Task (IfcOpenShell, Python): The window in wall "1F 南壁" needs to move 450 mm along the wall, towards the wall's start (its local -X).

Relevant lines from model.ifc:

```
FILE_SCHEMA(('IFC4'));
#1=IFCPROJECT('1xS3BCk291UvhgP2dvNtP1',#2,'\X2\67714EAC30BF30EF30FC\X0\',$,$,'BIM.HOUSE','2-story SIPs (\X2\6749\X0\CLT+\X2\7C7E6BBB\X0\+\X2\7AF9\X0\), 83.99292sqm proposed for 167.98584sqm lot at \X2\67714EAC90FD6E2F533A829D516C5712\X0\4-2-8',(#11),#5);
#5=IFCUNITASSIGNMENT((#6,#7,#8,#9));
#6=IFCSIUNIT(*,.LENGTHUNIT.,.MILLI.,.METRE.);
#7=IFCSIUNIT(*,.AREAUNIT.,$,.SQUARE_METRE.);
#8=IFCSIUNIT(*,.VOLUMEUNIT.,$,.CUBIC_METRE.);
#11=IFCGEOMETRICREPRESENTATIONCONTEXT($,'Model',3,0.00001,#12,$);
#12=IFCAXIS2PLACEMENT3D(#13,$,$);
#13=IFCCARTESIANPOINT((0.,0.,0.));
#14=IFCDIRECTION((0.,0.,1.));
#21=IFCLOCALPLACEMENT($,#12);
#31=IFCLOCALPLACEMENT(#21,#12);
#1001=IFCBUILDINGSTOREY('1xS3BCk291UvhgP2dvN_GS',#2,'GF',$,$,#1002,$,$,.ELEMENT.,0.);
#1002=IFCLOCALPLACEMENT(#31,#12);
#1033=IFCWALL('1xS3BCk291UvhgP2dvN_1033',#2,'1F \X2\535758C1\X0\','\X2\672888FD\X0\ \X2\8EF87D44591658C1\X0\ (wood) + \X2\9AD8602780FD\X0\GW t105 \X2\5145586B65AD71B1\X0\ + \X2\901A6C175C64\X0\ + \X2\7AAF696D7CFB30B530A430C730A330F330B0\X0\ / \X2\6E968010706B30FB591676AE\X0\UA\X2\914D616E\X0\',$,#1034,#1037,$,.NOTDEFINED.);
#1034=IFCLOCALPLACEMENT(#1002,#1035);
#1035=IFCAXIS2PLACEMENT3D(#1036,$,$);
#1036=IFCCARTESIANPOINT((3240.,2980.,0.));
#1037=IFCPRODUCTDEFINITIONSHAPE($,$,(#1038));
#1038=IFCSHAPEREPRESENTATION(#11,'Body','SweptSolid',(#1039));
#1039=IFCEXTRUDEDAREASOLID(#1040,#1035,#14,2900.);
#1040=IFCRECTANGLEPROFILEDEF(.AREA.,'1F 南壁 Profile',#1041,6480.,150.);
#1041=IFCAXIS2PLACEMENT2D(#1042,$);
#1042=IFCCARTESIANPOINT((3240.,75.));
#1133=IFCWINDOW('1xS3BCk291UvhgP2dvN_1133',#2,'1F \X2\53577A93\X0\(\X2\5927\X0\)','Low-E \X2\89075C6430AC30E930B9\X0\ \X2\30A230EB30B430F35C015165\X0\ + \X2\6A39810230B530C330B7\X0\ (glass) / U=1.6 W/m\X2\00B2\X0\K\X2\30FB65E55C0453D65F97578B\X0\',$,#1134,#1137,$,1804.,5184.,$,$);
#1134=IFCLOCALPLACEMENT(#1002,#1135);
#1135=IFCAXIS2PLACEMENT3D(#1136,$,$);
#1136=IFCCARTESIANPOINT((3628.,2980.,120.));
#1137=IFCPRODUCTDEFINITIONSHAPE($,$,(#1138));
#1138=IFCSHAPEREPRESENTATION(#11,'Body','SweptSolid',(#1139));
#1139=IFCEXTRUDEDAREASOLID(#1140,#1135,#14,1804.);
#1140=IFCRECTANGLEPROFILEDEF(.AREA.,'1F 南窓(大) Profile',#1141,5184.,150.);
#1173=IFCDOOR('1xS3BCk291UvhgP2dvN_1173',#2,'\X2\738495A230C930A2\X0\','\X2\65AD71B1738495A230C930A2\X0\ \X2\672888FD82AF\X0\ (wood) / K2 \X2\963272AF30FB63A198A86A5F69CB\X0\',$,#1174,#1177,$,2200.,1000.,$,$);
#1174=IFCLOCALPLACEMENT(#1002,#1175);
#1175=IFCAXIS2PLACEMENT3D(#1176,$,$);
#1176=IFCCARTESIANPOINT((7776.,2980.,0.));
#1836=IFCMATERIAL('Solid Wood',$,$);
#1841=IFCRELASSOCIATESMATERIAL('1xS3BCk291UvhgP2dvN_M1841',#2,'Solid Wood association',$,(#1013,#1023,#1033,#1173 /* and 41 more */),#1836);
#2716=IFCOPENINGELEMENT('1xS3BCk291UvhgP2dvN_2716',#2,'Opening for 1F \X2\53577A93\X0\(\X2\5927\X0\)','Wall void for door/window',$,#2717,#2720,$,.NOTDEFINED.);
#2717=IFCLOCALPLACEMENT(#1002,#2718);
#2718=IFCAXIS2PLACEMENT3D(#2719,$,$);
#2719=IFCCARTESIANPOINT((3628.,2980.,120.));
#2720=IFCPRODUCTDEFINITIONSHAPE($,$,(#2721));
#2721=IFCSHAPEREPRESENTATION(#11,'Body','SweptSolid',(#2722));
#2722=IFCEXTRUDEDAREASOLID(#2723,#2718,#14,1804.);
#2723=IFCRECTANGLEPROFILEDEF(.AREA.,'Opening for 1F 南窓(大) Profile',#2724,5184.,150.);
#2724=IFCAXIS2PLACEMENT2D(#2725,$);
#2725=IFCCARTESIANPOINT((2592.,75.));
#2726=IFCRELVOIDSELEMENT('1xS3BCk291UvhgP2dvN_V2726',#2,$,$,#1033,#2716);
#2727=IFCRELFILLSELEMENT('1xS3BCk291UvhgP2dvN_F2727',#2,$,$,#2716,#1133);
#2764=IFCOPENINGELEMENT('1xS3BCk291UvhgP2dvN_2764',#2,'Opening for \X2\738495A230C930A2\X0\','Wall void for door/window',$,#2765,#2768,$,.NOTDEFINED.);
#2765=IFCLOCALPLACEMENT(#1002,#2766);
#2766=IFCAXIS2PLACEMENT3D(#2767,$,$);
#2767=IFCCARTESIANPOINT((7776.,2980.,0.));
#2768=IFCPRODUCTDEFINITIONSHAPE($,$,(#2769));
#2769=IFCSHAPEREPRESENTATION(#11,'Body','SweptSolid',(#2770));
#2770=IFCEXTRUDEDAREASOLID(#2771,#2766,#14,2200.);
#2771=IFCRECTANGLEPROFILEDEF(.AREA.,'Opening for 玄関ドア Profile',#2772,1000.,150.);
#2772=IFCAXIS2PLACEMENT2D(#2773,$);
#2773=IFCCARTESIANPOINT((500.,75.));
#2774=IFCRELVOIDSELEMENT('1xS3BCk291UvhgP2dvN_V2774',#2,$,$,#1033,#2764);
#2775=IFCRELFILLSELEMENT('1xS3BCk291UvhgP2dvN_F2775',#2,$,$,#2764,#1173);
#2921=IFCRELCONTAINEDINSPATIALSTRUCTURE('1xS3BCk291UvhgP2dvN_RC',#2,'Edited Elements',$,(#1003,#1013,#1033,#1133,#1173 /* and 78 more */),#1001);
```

```python
import ifcopenshell
import ifcopenshell.api.geometry
import ifcopenshell.util.placement
import ifcopenshell.util.unit

model = ifcopenshell.open("model.ifc")
unit_scale = ifcopenshell.util.unit.calculate_unit_scale(model)

window = model.by_guid("1xS3BCk291UvhgP2dvN_1133")
opening = window.FillsVoids[0].RelatingOpeningElement
wall = opening.VoidsElements[0].RelatingBuildingElement

wall_matrix = ifcopenshell.util.placement.get_local_placement(wall.ObjectPlacement)
shift = wall_matrix[:3, 0] * -0.45 / unit_scale
before = ifcopenshell.util.placement.get_local_placement(window.ObjectPlacement)[:3, 3].copy()

# The window is not placed relative to its opening, so move both.
for product in (opening, window):
    matrix = ifcopenshell.util.placement.get_local_placement(product.ObjectPlacement)
    matrix[:3, 3] += shift
    ifcopenshell.api.geometry.edit_object_placement(model, product=product, matrix=matrix, is_si=False)

after = ifcopenshell.util.placement.get_local_placement(window.ObjectPlacement)[:3, 3]
print("window moved by", (after - before).round(3) + 0.0)

model.write("model_v2.ifc")
```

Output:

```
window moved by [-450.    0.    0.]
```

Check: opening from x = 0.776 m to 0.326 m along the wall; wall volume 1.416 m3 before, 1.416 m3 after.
